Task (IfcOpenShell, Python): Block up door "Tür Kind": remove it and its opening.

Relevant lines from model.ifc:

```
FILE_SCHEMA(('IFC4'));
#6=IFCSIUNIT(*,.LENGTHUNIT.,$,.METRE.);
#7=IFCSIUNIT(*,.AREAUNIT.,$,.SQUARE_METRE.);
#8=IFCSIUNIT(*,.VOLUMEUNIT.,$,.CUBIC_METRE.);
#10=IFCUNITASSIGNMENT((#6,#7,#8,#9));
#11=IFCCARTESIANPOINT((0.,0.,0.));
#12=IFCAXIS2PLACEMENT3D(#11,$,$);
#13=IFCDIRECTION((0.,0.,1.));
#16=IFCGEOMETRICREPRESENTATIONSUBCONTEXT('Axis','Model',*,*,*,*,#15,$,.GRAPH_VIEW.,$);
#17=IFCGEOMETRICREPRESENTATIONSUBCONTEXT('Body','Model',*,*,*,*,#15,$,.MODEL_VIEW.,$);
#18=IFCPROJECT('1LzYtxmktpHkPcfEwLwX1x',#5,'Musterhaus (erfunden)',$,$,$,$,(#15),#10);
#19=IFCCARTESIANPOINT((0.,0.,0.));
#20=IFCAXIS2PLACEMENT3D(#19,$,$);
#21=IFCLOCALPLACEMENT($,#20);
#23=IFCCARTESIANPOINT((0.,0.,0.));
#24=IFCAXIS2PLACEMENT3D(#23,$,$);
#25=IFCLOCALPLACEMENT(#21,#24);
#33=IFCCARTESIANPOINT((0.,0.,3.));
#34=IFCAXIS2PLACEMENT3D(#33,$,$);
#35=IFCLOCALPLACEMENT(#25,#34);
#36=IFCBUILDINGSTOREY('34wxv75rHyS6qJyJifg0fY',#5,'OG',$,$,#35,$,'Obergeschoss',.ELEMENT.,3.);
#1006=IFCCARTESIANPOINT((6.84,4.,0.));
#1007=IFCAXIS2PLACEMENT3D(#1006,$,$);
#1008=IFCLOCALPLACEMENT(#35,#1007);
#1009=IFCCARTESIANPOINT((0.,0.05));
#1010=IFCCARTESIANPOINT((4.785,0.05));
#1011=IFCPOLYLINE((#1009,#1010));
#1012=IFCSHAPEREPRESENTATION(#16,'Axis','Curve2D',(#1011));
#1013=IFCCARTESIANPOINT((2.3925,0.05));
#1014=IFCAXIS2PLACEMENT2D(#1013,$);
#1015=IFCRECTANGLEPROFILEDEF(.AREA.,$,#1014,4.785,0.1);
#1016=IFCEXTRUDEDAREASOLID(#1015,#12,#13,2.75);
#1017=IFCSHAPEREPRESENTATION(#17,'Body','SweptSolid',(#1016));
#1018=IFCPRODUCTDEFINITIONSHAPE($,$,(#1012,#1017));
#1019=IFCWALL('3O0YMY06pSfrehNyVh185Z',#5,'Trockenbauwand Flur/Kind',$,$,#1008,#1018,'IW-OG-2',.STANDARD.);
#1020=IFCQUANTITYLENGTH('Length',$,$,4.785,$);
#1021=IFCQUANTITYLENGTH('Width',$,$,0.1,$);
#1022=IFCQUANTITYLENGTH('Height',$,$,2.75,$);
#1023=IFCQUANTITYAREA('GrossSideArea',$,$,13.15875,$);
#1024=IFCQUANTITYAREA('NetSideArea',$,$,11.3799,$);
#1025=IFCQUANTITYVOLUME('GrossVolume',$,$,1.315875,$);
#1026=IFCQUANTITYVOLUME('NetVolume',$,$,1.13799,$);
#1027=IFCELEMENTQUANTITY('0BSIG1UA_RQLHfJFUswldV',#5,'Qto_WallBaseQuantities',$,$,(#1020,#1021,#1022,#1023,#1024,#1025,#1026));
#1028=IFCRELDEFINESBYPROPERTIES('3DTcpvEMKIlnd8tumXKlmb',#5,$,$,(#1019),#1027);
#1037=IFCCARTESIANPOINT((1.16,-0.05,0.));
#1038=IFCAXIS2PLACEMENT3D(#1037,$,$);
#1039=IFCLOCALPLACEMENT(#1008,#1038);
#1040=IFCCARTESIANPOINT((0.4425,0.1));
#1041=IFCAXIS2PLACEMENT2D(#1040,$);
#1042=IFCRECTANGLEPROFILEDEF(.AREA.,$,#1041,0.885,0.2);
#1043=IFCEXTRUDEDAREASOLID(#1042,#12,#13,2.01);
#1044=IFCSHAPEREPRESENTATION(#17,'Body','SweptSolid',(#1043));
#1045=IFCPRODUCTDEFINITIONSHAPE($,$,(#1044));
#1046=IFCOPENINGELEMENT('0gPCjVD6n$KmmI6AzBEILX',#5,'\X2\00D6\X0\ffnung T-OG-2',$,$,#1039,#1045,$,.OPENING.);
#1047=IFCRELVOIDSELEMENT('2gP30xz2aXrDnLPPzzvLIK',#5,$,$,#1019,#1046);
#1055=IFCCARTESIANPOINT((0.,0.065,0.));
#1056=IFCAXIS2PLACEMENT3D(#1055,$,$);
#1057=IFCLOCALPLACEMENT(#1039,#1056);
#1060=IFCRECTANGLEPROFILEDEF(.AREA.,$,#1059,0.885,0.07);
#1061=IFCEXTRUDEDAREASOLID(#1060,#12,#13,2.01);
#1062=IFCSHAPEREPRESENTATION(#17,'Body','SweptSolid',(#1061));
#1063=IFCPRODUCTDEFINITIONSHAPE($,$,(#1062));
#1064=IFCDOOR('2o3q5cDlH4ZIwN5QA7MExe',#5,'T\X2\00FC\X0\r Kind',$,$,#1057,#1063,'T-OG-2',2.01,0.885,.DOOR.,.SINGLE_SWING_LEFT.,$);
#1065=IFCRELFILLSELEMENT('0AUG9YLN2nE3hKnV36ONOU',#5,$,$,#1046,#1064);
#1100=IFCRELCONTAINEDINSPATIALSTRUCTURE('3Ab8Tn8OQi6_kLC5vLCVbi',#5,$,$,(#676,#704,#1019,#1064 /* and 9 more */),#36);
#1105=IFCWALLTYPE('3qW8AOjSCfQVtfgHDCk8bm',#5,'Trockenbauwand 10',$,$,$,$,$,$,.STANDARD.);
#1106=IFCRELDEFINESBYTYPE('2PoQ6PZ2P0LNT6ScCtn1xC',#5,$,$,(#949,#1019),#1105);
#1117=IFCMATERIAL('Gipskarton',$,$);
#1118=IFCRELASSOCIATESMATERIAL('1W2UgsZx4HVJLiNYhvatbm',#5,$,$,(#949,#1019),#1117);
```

```python
import ifcopenshell
import ifcopenshell.api.feature
import ifcopenshell.api.pset
import ifcopenshell.api.root
import ifcopenshell.geom
import ifcopenshell.util.element
import ifcopenshell.util.shape
import ifcopenshell.util.unit

model = ifcopenshell.open("model.ifc")
area_scale = ifcopenshell.util.unit.calculate_unit_scale(model, "AREAUNIT")
volume_scale = ifcopenshell.util.unit.calculate_unit_scale(model, "VOLUMEUNIT")
settings = ifcopenshell.geom.settings()


def volume(element):
    """Net volume in cubic metres, openings subtracted."""
    shape = ifcopenshell.geom.create_shape(settings, element)
    return ifcopenshell.util.shape.get_volume(shape.geometry)


door = model.by_id(1064)
opening = door.FillsVoids[0].RelatingOpeningElement
wall = opening.VoidsElements[0].RelatingBuildingElement
before = volume(wall)

ifcopenshell.api.root.remove_product(model, product=door)
ifcopenshell.api.feature.remove_feature(model, feature=opening)

after = volume(wall)
thickness = 0.1  # wall thickness in metres

# Update the wall's stored quantities.
qto = model.by_id(ifcopenshell.util.element.get_pset(wall, "Qto_WallBaseQuantities", should_inherit=False)["id"])
ifcopenshell.api.pset.edit_qto(model, qto=qto, properties={
    "NetSideArea": after / thickness / area_scale,
    "NetVolume": after / volume_scale,
})

print(f"wall volume {before:.3f} -> {after:.3f} m3")

model.write("model-out.ifc")
```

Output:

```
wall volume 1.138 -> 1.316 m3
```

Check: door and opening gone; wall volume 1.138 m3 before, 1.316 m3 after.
